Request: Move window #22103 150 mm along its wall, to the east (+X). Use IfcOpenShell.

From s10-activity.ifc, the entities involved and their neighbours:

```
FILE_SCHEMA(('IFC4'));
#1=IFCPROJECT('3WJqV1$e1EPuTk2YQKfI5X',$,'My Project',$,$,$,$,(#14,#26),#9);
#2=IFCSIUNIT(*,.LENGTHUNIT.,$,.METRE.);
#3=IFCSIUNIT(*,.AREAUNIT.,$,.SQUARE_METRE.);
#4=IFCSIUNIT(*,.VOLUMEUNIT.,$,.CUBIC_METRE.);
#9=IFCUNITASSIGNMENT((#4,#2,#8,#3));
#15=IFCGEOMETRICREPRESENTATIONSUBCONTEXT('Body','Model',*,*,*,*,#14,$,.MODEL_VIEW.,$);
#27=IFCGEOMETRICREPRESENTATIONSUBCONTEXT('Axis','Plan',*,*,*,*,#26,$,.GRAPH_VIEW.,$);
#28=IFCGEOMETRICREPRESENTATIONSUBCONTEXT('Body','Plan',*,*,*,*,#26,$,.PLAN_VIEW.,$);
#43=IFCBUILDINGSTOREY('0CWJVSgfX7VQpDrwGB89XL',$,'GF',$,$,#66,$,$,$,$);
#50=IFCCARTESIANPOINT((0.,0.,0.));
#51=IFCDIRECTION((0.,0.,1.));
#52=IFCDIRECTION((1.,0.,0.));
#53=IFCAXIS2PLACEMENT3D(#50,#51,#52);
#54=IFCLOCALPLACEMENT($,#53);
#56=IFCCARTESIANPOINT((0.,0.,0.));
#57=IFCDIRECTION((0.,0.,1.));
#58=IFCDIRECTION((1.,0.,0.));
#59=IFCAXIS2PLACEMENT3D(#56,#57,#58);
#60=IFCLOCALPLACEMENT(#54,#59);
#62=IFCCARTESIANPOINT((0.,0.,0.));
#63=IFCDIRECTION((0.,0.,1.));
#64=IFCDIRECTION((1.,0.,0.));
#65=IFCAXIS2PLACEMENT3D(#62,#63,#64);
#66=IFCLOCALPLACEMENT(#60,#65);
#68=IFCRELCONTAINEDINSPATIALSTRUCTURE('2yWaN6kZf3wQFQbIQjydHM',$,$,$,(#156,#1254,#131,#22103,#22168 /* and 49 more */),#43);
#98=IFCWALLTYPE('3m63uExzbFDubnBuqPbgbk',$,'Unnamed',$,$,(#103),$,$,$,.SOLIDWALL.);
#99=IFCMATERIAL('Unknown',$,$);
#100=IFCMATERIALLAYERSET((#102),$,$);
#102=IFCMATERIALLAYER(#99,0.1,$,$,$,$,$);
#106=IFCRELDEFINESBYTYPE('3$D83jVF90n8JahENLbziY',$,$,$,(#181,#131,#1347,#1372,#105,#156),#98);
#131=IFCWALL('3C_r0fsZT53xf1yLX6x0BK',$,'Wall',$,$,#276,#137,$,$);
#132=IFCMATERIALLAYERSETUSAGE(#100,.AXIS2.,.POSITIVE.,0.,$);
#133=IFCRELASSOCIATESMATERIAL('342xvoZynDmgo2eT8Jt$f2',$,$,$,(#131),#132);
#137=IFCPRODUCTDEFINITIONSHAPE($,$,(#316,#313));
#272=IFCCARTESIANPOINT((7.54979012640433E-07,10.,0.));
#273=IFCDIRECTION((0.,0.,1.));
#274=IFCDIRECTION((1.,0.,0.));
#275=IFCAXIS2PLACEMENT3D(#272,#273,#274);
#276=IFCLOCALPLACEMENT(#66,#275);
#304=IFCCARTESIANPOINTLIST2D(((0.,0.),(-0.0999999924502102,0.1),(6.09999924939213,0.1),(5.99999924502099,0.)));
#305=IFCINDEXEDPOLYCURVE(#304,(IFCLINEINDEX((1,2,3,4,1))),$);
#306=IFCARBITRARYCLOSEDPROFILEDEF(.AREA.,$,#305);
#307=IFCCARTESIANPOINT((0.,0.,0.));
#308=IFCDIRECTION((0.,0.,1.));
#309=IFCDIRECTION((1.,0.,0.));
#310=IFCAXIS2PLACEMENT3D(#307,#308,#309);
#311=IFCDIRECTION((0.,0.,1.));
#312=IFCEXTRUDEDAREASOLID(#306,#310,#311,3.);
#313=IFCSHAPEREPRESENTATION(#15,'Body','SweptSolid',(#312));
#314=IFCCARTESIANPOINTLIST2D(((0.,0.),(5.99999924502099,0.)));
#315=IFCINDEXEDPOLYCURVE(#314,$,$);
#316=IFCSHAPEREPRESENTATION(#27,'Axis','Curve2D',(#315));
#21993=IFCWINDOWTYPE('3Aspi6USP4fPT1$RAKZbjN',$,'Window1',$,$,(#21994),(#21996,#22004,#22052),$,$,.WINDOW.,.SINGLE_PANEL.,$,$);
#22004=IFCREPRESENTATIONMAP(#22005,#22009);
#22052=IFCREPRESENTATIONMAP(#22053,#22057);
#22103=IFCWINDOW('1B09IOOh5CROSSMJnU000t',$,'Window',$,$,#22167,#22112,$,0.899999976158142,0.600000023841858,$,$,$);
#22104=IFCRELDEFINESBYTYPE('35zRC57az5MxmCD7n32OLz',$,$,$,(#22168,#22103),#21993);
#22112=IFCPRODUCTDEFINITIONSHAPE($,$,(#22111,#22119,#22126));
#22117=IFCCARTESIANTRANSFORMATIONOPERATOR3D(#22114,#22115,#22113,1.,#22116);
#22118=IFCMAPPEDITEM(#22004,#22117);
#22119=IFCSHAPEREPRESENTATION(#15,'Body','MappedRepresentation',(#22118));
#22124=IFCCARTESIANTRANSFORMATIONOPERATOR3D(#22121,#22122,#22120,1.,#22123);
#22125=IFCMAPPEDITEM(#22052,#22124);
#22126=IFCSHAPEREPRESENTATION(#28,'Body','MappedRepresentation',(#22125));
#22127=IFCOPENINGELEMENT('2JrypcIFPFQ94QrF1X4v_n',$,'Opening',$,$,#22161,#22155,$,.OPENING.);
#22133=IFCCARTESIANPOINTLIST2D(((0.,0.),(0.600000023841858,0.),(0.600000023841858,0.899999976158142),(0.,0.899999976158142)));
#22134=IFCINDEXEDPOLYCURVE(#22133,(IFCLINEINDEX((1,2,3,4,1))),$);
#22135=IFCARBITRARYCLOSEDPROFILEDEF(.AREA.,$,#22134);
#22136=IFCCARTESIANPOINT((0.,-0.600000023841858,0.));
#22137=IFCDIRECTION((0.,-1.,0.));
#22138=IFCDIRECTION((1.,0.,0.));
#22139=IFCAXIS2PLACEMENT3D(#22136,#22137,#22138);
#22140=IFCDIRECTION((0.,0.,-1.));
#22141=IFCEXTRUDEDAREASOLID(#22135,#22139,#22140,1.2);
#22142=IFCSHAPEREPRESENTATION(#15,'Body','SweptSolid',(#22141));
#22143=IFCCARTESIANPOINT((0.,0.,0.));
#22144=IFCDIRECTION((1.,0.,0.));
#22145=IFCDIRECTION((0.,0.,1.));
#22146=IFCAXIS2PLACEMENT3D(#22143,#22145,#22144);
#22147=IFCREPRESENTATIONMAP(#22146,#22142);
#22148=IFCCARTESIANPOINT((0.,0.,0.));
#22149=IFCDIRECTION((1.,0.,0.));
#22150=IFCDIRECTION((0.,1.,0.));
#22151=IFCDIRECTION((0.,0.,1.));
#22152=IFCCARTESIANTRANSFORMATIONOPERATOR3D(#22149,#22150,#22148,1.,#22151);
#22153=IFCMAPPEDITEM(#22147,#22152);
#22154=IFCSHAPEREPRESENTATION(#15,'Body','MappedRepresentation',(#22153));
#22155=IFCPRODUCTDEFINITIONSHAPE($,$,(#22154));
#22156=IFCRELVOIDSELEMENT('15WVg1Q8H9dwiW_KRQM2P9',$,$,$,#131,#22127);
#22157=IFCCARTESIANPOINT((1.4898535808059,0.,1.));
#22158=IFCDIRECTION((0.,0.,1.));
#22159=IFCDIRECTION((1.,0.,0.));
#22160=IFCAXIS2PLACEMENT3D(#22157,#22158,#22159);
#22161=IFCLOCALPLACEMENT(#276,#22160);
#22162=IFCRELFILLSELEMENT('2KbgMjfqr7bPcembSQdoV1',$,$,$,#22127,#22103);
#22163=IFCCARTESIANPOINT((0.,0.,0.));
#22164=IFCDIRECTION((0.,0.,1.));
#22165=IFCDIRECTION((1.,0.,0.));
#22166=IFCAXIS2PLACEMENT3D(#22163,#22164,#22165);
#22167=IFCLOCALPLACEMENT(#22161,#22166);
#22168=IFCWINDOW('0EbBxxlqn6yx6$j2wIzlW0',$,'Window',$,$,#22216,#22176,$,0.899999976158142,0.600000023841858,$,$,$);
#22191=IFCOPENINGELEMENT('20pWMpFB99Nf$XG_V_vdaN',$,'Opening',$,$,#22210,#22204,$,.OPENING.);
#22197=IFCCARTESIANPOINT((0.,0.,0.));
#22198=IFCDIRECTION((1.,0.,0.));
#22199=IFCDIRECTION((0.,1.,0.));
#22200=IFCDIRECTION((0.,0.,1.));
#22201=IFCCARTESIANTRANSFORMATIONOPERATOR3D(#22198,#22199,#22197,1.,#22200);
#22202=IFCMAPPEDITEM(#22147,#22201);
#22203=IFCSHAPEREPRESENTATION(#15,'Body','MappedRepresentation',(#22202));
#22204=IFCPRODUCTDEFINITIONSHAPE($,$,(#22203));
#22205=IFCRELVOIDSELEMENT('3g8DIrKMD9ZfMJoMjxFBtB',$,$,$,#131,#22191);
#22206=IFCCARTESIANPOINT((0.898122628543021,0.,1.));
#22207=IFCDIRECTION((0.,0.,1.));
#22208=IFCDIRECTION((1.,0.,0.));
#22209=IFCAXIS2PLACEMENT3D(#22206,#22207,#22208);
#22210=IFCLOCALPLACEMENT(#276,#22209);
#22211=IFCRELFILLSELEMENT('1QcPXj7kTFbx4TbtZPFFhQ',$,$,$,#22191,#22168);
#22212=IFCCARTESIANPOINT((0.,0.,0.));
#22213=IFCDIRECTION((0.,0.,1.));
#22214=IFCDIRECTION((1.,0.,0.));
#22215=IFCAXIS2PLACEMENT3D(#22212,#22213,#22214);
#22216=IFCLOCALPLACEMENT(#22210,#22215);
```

```python
import ifcopenshell
import ifcopenshell.api.geometry
import ifcopenshell.util.placement
import ifcopenshell.util.unit

model = ifcopenshell.open("s10-activity.ifc")
unit_scale = ifcopenshell.util.unit.calculate_unit_scale(model)

window = model.by_guid("1B09IOOh5CROSSMJnU000t")
opening = window.FillsVoids[0].RelatingOpeningElement
wall = opening.VoidsElements[0].RelatingBuildingElement

wall_matrix = ifcopenshell.util.placement.get_local_placement(wall.ObjectPlacement)
shift = wall_matrix[:3, 0] * 0.15 / unit_scale
before = ifcopenshell.util.placement.get_local_placement(window.ObjectPlacement)[:3, 3].copy()

# The window is placed relative to its opening, so it follows when the opening moves.
matrix = ifcopenshell.util.placement.get_local_placement(opening.ObjectPlacement)
matrix[:3, 3] += shift
ifcopenshell.api.geometry.edit_object_placement(
    model, product=opening, matrix=matrix, is_si=False, should_transform_children=True
)

after = ifcopenshell.util.placement.get_local_placement(window.ObjectPlacement)[:3, 3]
print("window moved by", (after - before).round(3) + 0.0)

model.write("s10-activity_v2.ifc")
```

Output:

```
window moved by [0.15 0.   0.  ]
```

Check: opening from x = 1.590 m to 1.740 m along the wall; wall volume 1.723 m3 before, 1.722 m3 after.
